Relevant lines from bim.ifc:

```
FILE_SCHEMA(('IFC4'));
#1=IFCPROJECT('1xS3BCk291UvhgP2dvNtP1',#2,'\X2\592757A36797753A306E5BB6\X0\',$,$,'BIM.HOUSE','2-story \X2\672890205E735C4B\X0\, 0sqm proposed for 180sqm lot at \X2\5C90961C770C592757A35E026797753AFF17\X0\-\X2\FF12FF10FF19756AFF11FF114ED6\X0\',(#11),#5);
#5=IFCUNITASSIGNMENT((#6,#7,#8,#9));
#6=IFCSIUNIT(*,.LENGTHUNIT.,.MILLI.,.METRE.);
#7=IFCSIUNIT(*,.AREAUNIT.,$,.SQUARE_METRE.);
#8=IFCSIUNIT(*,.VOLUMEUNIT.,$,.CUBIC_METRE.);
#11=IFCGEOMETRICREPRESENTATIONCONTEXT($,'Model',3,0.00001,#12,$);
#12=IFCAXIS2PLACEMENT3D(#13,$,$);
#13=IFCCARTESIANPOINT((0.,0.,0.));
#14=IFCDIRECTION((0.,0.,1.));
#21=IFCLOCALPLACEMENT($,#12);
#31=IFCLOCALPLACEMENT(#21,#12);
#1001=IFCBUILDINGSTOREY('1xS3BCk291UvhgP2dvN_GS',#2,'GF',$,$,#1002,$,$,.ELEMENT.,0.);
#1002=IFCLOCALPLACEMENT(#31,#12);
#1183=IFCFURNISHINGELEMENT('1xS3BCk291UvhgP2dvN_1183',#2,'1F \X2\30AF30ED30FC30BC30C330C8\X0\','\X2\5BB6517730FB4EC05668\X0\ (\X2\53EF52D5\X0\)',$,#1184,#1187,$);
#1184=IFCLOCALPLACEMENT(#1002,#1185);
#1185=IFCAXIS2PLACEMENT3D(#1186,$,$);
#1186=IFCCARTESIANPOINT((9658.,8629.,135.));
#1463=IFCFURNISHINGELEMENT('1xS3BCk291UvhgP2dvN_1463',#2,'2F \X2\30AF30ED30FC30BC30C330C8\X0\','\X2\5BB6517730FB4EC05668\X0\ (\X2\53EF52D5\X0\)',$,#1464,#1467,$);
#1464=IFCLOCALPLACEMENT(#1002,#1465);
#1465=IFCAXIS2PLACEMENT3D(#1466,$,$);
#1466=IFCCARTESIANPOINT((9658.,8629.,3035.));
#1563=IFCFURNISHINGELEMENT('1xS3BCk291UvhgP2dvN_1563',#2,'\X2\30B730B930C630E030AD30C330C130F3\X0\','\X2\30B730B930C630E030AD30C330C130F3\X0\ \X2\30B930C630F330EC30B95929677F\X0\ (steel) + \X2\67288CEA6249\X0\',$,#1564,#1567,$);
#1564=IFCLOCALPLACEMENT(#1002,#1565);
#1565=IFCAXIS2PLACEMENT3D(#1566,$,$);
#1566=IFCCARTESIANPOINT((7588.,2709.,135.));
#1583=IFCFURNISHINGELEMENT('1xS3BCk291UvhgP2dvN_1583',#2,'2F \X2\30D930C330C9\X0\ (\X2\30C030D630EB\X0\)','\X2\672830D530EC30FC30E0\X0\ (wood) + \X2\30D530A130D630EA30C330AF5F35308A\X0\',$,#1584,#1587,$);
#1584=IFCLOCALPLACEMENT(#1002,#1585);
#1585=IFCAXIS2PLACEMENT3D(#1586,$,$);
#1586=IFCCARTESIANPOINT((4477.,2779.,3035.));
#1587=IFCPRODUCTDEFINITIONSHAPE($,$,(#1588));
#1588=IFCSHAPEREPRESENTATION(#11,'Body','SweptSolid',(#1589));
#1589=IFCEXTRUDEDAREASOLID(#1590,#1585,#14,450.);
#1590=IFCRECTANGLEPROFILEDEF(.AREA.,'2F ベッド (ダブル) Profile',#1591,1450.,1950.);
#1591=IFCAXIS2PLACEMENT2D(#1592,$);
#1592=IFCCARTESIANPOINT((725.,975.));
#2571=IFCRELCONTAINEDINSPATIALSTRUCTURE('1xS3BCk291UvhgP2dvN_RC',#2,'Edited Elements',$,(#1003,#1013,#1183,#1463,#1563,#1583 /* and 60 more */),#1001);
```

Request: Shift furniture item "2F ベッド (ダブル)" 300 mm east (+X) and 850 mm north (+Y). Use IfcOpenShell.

```python
import ifcopenshell
import ifcopenshell.api.geometry
import ifcopenshell.util.placement
import ifcopenshell.util.unit

model = ifcopenshell.open("bim.ifc")
unit_scale = ifcopenshell.util.unit.calculate_unit_scale(model)

item = model.by_guid("1xS3BCk291UvhgP2dvN_1583")
matrix = ifcopenshell.util.placement.get_local_placement(item.ObjectPlacement)
matrix[0, 3] += 0.3 / unit_scale
matrix[1, 3] += 0.85 / unit_scale
ifcopenshell.api.geometry.edit_object_placement(model, product=item, matrix=matrix, is_si=False)

print(ifcopenshell.util.placement.get_local_placement(item.ObjectPlacement).round(3) + 0.0)

model.write("bim_rev.ifc")
```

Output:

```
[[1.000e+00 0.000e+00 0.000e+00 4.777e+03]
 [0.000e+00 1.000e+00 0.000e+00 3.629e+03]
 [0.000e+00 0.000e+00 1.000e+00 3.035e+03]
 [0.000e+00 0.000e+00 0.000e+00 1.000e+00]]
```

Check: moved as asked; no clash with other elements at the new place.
